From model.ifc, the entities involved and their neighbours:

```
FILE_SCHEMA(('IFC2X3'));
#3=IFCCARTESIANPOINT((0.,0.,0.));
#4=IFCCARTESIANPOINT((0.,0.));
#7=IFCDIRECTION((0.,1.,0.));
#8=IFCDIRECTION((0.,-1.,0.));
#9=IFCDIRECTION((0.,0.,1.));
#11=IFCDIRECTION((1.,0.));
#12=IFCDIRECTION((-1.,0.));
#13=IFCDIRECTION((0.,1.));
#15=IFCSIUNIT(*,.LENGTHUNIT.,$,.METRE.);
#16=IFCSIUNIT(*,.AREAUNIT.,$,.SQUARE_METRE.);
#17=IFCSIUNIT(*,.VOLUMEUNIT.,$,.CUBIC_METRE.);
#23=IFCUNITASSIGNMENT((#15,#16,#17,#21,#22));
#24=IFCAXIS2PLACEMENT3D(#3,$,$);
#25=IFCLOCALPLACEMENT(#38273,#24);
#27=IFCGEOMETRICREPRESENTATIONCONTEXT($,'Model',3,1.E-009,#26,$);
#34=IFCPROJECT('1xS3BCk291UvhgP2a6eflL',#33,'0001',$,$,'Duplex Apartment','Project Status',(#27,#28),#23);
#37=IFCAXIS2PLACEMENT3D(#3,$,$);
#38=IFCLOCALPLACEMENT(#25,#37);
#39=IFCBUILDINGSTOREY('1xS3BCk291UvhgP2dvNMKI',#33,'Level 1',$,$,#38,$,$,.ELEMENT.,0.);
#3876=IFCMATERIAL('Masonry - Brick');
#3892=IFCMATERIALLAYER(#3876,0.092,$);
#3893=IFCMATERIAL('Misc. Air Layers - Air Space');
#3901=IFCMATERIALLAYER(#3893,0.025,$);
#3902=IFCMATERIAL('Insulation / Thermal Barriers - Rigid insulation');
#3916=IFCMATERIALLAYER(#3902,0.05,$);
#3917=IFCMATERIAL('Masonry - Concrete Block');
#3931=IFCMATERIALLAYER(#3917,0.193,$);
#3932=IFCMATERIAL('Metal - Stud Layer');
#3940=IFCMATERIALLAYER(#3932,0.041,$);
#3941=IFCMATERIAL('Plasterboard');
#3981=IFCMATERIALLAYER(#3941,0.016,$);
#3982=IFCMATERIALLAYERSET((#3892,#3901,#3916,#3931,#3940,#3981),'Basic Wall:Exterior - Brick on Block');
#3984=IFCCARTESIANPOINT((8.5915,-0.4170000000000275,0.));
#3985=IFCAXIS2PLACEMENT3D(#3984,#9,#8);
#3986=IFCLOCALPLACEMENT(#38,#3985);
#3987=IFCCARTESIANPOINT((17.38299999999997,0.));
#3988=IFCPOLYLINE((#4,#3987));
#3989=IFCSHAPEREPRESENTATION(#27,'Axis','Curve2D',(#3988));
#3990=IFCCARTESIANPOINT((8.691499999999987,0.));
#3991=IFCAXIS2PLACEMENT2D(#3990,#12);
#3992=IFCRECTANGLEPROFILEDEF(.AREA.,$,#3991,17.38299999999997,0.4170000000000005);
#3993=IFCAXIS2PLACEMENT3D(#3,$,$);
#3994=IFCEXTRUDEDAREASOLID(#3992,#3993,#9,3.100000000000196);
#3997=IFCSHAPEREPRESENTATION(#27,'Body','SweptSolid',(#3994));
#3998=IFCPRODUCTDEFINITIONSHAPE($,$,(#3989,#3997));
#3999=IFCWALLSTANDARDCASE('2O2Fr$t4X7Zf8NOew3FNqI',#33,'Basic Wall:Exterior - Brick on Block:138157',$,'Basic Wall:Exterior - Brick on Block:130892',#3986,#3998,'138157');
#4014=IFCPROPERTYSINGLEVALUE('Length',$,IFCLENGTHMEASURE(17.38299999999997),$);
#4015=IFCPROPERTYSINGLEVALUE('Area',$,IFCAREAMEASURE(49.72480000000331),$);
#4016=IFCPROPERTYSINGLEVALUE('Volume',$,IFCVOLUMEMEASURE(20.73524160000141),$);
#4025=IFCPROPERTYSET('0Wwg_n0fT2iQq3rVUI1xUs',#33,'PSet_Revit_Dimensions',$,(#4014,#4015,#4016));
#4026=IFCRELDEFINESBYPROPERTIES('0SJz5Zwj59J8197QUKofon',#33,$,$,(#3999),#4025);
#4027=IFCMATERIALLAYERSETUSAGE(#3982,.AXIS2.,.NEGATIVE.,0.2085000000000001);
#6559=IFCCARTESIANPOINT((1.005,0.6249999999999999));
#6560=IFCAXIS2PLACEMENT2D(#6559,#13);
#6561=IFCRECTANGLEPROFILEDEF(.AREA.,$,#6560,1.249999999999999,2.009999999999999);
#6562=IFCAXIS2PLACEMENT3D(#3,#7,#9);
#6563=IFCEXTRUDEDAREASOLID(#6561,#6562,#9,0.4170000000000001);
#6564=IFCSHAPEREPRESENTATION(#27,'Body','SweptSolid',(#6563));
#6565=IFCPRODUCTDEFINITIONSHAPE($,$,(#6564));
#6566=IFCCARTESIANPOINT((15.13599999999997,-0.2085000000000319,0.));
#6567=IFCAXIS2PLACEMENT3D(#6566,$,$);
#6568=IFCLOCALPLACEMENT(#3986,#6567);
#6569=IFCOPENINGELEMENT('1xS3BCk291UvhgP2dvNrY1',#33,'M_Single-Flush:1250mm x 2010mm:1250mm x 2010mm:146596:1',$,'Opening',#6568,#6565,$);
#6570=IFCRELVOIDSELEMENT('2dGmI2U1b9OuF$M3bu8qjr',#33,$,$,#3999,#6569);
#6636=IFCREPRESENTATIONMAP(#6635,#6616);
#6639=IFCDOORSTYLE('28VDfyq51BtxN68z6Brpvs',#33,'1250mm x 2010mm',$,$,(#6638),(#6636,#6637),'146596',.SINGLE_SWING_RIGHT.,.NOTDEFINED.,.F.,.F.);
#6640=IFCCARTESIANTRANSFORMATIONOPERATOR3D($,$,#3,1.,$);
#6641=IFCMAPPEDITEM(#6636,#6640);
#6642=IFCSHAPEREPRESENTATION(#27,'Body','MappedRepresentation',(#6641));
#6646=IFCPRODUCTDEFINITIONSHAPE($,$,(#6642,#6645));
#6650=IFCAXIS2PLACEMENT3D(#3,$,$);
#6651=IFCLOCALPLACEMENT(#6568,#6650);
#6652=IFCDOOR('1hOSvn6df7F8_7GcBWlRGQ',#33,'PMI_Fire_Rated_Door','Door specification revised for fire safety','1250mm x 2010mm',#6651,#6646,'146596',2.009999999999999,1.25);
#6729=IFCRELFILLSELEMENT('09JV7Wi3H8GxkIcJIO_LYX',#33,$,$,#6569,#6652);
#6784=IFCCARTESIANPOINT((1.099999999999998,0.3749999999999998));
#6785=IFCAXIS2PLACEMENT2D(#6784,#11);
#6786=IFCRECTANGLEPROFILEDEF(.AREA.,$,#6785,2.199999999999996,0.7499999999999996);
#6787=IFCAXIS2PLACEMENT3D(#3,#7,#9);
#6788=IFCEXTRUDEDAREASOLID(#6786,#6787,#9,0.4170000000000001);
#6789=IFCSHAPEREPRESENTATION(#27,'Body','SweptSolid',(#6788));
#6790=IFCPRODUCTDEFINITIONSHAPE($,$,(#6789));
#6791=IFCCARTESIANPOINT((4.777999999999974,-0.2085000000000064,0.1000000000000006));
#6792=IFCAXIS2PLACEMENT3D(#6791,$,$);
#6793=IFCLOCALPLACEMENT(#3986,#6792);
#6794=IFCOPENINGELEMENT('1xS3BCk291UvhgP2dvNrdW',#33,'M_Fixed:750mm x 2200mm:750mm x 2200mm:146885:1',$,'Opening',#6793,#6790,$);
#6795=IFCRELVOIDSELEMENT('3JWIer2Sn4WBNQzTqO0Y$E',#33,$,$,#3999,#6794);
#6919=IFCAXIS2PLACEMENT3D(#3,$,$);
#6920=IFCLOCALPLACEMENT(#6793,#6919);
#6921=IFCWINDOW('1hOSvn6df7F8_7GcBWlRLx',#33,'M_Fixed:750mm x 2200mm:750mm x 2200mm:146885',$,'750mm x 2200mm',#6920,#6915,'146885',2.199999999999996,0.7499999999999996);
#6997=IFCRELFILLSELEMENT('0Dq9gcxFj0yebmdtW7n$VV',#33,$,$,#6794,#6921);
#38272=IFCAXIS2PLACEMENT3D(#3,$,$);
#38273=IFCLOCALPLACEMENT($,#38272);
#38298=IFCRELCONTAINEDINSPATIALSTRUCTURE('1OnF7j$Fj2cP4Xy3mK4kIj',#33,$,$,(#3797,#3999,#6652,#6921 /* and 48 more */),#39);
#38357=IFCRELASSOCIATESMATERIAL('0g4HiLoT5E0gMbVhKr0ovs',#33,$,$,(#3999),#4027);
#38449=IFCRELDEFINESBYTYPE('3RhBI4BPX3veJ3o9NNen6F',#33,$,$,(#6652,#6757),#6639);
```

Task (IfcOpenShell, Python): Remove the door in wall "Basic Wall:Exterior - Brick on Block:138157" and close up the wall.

```python
import ifcopenshell
import ifcopenshell.api.feature
import ifcopenshell.api.pset
import ifcopenshell.api.root
import ifcopenshell.geom
import ifcopenshell.util.element
import ifcopenshell.util.shape
import ifcopenshell.util.unit

model = ifcopenshell.open("model.ifc")
area_scale = ifcopenshell.util.unit.calculate_unit_scale(model, "AREAUNIT")
volume_scale = ifcopenshell.util.unit.calculate_unit_scale(model, "VOLUMEUNIT")
settings = ifcopenshell.geom.settings()


def volume(element):
    """Net volume in cubic metres, openings subtracted."""
    shape = ifcopenshell.geom.create_shape(settings, element)
    return ifcopenshell.util.shape.get_volume(shape.geometry)


door = model.by_id(6652)
opening = door.FillsVoids[0].RelatingOpeningElement
wall = opening.VoidsElements[0].RelatingBuildingElement
before = volume(wall)

ifcopenshell.api.root.remove_product(model, product=door)
ifcopenshell.api.feature.remove_feature(model, feature=opening)

after = volume(wall)
thickness = 0.417  # wall thickness in metres

# Update the wall's stored quantities.
pset = model.by_id(ifcopenshell.util.element.get_pset(wall, "PSet_Revit_Dimensions", should_inherit=False)["id"])
ifcopenshell.api.pset.edit_pset(model, pset=pset, properties={
    "Area": model.create_entity("IfcAreaMeasure", after / thickness / area_scale),
    "Volume": model.create_entity("IfcVolumeMeasure", after / volume_scale),
})

print(f"wall volume {before:.3f} -> {after:.3f} m3")

model.write("model-out.ifc")
```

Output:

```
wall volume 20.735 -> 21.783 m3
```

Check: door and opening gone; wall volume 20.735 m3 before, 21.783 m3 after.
